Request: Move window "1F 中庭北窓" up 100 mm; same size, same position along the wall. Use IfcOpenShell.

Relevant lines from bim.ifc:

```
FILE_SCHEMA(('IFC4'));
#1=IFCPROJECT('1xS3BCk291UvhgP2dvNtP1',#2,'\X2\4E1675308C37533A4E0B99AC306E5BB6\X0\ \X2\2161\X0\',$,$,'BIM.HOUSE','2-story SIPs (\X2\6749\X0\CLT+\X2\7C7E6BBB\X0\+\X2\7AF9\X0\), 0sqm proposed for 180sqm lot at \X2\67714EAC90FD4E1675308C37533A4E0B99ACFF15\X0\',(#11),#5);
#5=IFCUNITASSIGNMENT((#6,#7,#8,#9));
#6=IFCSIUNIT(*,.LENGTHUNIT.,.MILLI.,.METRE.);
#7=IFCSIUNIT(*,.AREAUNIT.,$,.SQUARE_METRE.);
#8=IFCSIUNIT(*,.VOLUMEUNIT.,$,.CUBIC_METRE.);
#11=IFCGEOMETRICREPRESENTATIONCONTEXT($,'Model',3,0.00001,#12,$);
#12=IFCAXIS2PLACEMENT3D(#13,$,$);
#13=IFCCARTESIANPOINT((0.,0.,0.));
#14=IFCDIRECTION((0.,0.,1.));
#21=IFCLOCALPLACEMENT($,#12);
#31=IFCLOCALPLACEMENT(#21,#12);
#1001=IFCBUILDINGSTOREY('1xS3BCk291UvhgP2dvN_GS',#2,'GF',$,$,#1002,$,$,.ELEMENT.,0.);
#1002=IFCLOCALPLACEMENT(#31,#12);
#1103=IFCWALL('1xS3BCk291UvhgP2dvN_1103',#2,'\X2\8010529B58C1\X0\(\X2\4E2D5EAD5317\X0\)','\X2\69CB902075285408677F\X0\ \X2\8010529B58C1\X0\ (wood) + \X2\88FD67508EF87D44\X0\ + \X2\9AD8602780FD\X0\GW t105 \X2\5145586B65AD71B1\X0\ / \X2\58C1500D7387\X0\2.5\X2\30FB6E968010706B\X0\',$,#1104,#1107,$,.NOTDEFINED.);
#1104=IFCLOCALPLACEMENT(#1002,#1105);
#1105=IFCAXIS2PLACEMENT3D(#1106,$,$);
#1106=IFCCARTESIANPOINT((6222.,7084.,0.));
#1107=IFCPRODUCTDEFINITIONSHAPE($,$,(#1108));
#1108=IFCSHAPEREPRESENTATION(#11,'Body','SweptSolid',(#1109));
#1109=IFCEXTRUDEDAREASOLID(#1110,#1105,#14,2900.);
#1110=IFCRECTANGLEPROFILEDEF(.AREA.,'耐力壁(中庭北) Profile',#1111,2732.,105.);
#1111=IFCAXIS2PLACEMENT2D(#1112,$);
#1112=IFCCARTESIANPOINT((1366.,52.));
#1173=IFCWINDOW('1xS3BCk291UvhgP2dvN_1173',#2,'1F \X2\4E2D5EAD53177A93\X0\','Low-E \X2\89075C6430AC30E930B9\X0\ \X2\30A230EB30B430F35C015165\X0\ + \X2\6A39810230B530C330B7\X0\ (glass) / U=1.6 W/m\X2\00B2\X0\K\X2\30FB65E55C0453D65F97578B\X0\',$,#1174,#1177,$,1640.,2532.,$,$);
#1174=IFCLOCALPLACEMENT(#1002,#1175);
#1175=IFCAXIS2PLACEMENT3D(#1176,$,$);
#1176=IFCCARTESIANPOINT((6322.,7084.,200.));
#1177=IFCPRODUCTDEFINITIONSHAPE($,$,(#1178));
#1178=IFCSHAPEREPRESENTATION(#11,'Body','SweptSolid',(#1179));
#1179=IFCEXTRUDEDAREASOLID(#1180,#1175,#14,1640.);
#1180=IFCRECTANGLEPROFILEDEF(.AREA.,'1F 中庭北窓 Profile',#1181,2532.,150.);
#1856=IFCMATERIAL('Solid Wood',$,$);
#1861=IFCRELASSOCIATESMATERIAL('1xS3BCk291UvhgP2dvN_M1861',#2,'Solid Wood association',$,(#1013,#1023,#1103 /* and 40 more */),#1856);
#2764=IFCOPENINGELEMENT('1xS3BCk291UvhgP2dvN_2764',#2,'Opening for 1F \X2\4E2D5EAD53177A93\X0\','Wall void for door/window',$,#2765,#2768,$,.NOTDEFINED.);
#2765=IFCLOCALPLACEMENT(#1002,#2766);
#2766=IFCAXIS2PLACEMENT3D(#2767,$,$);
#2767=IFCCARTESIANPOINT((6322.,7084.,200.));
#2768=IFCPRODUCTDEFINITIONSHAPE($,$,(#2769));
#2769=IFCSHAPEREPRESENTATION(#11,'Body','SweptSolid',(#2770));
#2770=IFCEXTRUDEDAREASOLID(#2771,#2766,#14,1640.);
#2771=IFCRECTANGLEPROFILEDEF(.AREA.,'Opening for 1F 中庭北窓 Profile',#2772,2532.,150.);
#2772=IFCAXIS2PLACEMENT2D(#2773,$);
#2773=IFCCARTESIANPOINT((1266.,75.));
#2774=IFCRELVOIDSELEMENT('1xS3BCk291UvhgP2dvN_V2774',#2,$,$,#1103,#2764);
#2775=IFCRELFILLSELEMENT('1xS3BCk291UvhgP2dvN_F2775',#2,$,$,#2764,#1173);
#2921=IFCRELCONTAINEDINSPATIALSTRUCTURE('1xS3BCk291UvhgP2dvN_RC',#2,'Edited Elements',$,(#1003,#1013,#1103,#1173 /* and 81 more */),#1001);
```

```python
import numpy as np
import ifcopenshell
import ifcopenshell.api.geometry
import ifcopenshell.util.placement
import ifcopenshell.util.unit

model = ifcopenshell.open("bim.ifc")
unit_scale = ifcopenshell.util.unit.calculate_unit_scale(model)

window = model.by_id(1173)
opening = window.FillsVoids[0].RelatingOpeningElement
dz = 0.1 / unit_scale

shift = np.array([0.0, 0.0, dz])
# The window is not placed relative to its opening, so move both.
for product in (opening, window):
    matrix = ifcopenshell.util.placement.get_local_placement(product.ObjectPlacement)
    matrix[:3, 3] += shift
    ifcopenshell.api.geometry.edit_object_placement(model, product=product, matrix=matrix, is_si=False)

print(f"moved by {dz * unit_scale:+.3f} m")

model.write("bim_updated.ifc")
```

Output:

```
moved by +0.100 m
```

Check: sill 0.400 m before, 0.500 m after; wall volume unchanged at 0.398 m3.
